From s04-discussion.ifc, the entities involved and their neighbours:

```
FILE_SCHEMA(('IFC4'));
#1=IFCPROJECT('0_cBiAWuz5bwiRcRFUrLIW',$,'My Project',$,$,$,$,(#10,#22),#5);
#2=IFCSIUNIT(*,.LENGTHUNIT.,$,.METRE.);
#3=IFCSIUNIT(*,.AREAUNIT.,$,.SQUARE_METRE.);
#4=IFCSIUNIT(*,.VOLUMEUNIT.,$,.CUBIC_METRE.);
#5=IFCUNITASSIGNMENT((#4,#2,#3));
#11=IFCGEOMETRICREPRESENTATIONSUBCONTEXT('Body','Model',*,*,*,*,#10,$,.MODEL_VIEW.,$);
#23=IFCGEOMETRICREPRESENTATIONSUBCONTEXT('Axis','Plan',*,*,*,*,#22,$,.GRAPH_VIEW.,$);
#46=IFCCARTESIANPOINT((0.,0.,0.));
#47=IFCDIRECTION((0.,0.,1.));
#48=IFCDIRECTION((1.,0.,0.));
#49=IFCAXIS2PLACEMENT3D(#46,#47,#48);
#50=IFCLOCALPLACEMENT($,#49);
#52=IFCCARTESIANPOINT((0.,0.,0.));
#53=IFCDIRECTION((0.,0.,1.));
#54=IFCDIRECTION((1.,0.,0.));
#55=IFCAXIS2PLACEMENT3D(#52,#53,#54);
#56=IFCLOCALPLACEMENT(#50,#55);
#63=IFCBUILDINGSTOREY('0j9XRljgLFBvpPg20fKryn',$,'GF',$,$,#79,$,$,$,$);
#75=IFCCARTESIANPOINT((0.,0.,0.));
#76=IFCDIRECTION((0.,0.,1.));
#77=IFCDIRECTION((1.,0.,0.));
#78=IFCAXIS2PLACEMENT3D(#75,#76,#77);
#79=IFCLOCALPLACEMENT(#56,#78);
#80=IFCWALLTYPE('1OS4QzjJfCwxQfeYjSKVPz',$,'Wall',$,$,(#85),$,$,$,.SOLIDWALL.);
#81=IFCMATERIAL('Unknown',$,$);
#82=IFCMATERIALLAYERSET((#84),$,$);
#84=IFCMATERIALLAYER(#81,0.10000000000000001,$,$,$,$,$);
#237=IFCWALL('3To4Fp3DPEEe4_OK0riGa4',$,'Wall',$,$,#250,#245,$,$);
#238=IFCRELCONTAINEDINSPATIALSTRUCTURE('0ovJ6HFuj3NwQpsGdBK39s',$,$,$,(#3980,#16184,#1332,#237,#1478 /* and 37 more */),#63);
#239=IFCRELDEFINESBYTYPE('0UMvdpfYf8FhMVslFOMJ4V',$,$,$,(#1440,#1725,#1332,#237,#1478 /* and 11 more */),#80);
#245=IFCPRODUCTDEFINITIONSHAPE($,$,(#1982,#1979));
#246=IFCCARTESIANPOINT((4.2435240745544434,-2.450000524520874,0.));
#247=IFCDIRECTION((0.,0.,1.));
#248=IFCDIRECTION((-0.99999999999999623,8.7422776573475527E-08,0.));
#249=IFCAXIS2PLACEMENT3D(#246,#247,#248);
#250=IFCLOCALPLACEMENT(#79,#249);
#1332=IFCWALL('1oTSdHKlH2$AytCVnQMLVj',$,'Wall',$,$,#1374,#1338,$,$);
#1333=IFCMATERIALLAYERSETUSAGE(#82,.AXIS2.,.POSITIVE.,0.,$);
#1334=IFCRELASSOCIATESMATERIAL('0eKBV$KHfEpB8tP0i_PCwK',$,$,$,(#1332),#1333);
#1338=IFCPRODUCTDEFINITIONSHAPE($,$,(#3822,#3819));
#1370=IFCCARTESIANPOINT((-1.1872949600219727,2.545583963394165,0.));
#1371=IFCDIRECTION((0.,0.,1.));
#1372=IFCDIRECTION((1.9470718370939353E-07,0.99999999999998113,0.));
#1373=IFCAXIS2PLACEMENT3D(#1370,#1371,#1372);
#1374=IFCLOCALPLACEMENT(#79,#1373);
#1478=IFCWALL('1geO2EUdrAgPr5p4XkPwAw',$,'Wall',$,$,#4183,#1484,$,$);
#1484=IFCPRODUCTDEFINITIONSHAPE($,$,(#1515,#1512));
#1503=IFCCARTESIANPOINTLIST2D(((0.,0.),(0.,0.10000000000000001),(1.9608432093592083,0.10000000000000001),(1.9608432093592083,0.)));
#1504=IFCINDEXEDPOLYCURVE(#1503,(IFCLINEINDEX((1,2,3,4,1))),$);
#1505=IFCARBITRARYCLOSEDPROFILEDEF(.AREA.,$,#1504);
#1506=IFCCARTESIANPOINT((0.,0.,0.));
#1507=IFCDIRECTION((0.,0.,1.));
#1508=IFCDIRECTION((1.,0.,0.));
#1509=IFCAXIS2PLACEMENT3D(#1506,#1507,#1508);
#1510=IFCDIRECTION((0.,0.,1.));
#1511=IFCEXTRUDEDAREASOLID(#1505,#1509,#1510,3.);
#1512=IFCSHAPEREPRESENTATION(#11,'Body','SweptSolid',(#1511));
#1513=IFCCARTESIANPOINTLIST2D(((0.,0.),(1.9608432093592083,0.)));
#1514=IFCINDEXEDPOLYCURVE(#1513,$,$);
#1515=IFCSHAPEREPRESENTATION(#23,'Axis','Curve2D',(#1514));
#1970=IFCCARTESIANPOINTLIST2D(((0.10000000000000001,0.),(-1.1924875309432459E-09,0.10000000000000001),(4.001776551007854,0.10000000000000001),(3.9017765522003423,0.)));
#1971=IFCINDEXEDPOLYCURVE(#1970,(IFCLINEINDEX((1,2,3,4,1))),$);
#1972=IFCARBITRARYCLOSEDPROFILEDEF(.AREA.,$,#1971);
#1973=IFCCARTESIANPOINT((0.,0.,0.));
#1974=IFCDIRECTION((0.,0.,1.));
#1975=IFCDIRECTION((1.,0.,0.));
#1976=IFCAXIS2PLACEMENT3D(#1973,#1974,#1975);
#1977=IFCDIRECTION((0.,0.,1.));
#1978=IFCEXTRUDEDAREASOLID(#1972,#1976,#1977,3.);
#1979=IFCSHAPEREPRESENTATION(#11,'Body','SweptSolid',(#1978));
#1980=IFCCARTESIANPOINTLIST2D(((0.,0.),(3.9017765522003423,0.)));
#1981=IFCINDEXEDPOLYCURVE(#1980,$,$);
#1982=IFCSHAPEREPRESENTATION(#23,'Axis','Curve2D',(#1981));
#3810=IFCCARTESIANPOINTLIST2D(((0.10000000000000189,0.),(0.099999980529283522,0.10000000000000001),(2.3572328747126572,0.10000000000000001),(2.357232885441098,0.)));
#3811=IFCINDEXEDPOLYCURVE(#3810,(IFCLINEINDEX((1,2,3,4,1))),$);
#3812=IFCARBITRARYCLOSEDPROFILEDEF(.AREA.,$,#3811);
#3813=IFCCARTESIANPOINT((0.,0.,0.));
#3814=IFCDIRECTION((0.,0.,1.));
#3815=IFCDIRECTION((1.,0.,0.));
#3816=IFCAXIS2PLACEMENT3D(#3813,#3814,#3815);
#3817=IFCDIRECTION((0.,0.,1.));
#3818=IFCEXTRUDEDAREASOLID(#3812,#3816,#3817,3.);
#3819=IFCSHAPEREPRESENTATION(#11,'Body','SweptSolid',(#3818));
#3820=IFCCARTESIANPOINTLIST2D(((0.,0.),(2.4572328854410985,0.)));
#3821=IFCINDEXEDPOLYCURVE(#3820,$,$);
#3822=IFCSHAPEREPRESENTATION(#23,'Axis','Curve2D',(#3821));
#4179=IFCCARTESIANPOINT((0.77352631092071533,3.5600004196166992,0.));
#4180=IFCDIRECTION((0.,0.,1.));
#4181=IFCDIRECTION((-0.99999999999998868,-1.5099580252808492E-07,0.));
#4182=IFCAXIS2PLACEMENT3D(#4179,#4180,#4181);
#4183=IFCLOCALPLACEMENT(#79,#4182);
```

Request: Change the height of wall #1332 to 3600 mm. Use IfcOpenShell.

```python
import ifcopenshell
import ifcopenshell.geom
import ifcopenshell.util.representation
import ifcopenshell.util.shape
import ifcopenshell.util.unit

model = ifcopenshell.open("s04-discussion.ifc")
unit_scale = ifcopenshell.util.unit.calculate_unit_scale(model)
settings = ifcopenshell.geom.settings()


def volume(element):
    """Net volume in cubic metres, openings subtracted."""
    shape = ifcopenshell.geom.create_shape(settings, element)
    return ifcopenshell.util.shape.get_volume(shape.geometry)


wall = model.by_guid("1oTSdHKlH2$AytCVnQMLVj")
before = volume(wall)

body = ifcopenshell.util.representation.get_representation(wall, "Model", "Body")
solid = body.Items[0]
old_height = solid.Depth
solid.Depth = 3.6 / unit_scale
after = volume(wall)

print(f"height {old_height:g} -> {solid.Depth:g}, volume {before:.3f} -> {after:.3f} m3")

model.write("s04-discussion_updated.ifc")
```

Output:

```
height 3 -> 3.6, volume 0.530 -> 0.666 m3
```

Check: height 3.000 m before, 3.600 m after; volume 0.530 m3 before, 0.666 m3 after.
